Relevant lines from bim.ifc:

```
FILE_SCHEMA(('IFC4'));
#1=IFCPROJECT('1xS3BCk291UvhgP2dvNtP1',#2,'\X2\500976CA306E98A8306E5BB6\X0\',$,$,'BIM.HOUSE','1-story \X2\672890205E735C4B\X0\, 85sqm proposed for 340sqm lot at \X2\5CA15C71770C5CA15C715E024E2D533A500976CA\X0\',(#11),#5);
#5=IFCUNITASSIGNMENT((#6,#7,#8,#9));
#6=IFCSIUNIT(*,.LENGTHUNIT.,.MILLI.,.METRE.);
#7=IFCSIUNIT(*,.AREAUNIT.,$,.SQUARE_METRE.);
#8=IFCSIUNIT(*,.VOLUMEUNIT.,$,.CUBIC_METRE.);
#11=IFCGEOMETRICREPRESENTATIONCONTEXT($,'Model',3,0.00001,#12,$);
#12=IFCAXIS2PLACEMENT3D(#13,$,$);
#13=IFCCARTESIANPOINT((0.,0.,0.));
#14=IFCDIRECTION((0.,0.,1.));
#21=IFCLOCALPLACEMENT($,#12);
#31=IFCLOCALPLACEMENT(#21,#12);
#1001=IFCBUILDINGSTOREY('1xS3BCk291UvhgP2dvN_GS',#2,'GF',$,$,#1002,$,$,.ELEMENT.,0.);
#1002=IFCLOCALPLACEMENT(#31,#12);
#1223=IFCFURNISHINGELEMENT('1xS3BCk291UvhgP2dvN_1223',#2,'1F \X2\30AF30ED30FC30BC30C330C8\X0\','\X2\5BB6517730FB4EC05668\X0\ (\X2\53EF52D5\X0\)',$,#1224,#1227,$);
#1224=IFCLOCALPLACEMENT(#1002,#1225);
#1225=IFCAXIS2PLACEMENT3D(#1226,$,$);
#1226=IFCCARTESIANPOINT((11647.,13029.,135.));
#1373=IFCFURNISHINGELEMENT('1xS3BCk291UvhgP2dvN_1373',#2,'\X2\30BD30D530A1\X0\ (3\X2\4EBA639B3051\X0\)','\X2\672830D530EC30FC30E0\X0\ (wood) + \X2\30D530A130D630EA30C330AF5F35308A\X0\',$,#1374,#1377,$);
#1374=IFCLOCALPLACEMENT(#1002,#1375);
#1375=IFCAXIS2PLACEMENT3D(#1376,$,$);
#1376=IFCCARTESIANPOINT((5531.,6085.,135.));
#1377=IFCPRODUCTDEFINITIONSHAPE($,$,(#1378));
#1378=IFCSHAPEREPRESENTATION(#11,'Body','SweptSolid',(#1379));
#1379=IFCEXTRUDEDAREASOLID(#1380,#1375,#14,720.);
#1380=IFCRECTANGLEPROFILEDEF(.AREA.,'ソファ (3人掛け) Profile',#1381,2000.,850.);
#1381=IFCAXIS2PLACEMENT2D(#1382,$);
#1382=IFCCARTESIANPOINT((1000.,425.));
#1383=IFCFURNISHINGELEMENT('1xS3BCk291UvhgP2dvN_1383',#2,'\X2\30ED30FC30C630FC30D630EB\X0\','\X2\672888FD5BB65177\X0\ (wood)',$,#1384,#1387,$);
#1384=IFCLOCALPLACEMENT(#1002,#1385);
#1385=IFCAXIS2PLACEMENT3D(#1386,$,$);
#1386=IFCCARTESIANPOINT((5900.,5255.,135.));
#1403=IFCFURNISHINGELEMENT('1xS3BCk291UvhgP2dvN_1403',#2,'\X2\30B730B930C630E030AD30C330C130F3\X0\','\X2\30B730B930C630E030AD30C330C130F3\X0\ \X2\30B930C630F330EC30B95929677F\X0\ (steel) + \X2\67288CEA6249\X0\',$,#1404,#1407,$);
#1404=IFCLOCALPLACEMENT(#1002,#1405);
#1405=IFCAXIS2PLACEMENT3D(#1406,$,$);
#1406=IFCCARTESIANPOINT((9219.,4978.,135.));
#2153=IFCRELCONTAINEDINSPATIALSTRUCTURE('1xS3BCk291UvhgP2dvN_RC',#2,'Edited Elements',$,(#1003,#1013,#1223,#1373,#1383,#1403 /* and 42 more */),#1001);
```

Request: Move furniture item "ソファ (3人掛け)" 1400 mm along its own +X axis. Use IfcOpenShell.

```python
import ifcopenshell
import ifcopenshell.api.geometry
import ifcopenshell.util.placement
import ifcopenshell.util.unit

model = ifcopenshell.open("bim.ifc")
unit_scale = ifcopenshell.util.unit.calculate_unit_scale(model)

item = model.by_guid("1xS3BCk291UvhgP2dvN_1373")
matrix = ifcopenshell.util.placement.get_local_placement(item.ObjectPlacement)
matrix[:3, 3] += matrix[:3, 0] * 1.4 / unit_scale
ifcopenshell.api.geometry.edit_object_placement(model, product=item, matrix=matrix, is_si=False)

print(ifcopenshell.util.placement.get_local_placement(item.ObjectPlacement).round(3) + 0.0)

model.write("bim_updated.ifc")
```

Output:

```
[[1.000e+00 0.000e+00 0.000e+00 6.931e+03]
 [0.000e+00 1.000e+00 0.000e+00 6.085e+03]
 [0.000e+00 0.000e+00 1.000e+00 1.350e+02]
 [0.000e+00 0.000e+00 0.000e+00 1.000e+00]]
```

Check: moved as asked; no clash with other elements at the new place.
